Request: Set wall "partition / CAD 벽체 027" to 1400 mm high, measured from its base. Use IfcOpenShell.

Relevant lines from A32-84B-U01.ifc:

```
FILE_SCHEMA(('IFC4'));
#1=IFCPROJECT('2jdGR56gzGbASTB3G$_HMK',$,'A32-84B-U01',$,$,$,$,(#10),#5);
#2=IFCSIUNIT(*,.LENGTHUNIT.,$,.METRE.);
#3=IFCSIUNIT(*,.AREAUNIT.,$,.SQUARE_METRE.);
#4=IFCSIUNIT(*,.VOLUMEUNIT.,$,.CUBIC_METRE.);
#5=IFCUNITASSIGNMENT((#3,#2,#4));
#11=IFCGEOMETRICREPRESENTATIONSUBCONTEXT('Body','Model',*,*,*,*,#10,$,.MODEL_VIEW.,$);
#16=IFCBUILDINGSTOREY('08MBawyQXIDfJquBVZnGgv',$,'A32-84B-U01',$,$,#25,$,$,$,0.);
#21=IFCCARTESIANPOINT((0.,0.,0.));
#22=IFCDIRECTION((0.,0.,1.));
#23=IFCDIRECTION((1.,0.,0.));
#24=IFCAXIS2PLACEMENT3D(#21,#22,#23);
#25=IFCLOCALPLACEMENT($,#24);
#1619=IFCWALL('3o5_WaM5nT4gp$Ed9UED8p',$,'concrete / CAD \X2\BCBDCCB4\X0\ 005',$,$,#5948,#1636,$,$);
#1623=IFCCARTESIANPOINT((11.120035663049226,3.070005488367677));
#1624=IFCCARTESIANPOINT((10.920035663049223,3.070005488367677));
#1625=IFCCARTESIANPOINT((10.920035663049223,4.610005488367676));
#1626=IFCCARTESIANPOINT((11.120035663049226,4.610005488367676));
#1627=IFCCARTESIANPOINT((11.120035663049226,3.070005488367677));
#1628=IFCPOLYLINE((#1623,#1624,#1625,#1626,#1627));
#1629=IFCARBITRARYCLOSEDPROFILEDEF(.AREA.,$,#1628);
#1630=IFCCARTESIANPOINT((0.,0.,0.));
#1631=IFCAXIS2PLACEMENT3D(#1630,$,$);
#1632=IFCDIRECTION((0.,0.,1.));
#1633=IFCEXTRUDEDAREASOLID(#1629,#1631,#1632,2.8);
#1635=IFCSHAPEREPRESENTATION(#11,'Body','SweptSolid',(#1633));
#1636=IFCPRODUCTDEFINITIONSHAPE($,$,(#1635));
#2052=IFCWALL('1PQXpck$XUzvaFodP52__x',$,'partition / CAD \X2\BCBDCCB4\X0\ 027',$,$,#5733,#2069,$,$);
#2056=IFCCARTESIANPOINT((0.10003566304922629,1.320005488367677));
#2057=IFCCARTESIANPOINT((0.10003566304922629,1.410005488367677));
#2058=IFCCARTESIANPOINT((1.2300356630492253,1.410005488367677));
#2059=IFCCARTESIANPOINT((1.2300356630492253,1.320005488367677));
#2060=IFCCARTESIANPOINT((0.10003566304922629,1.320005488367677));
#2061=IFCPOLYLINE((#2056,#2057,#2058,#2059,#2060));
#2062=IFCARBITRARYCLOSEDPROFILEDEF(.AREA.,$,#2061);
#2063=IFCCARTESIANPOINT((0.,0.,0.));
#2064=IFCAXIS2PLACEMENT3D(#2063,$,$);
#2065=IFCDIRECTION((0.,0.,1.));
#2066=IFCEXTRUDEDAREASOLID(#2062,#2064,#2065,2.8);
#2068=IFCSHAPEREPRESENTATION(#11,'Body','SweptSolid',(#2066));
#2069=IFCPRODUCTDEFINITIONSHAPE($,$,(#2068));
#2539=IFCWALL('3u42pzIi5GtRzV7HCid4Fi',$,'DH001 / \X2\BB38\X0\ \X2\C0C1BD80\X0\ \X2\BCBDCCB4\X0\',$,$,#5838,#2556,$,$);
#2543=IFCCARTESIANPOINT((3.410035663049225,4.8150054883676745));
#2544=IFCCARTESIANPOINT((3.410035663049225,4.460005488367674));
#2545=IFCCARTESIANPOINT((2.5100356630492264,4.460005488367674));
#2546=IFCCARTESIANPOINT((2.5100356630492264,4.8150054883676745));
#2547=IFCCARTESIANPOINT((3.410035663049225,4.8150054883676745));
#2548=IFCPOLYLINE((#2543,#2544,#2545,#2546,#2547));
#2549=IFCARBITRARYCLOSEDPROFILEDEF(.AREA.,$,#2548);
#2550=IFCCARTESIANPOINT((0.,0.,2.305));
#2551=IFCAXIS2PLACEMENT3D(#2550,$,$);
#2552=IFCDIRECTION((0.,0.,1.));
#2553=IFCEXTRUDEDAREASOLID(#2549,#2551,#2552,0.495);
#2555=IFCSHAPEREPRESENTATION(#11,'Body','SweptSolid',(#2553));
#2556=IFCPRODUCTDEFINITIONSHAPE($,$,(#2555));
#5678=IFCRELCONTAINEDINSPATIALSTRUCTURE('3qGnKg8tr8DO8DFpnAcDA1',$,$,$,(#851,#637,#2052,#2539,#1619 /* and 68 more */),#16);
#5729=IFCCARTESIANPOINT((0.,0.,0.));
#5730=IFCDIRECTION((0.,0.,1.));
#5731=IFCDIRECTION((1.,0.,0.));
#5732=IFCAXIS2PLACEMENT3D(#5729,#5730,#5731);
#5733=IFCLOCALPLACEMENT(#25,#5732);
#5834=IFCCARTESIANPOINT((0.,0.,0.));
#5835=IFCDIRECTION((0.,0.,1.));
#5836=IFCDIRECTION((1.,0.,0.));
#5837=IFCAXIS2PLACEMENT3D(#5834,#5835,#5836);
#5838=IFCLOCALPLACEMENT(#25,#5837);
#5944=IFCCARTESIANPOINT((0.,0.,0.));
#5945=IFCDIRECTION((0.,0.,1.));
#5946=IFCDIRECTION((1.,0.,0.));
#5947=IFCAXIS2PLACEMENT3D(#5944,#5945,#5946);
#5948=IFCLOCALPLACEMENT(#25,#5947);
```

```python
import ifcopenshell
import ifcopenshell.geom
import ifcopenshell.util.representation
import ifcopenshell.util.shape

model = ifcopenshell.open("A32-84B-U01.ifc")
settings = ifcopenshell.geom.settings()


def volume(element):
    """Net volume in cubic metres, openings subtracted."""
    shape = ifcopenshell.geom.create_shape(settings, element)
    return ifcopenshell.util.shape.get_volume(shape.geometry)


wall = model.by_guid("1PQXpck$XUzvaFodP52__x")
before = volume(wall)

body = ifcopenshell.util.representation.get_representation(wall, "Model", "Body")
solid = body.Items[0]
old_height = solid.Depth
solid.Depth = 1.4
after = volume(wall)

print(f"height {old_height:g} -> {solid.Depth:g}, volume {before:.3f} -> {after:.3f} m3")

model.write("A32-84B-U01_edited.ifc")
```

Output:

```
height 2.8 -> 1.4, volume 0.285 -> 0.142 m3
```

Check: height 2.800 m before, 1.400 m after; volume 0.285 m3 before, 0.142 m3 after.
